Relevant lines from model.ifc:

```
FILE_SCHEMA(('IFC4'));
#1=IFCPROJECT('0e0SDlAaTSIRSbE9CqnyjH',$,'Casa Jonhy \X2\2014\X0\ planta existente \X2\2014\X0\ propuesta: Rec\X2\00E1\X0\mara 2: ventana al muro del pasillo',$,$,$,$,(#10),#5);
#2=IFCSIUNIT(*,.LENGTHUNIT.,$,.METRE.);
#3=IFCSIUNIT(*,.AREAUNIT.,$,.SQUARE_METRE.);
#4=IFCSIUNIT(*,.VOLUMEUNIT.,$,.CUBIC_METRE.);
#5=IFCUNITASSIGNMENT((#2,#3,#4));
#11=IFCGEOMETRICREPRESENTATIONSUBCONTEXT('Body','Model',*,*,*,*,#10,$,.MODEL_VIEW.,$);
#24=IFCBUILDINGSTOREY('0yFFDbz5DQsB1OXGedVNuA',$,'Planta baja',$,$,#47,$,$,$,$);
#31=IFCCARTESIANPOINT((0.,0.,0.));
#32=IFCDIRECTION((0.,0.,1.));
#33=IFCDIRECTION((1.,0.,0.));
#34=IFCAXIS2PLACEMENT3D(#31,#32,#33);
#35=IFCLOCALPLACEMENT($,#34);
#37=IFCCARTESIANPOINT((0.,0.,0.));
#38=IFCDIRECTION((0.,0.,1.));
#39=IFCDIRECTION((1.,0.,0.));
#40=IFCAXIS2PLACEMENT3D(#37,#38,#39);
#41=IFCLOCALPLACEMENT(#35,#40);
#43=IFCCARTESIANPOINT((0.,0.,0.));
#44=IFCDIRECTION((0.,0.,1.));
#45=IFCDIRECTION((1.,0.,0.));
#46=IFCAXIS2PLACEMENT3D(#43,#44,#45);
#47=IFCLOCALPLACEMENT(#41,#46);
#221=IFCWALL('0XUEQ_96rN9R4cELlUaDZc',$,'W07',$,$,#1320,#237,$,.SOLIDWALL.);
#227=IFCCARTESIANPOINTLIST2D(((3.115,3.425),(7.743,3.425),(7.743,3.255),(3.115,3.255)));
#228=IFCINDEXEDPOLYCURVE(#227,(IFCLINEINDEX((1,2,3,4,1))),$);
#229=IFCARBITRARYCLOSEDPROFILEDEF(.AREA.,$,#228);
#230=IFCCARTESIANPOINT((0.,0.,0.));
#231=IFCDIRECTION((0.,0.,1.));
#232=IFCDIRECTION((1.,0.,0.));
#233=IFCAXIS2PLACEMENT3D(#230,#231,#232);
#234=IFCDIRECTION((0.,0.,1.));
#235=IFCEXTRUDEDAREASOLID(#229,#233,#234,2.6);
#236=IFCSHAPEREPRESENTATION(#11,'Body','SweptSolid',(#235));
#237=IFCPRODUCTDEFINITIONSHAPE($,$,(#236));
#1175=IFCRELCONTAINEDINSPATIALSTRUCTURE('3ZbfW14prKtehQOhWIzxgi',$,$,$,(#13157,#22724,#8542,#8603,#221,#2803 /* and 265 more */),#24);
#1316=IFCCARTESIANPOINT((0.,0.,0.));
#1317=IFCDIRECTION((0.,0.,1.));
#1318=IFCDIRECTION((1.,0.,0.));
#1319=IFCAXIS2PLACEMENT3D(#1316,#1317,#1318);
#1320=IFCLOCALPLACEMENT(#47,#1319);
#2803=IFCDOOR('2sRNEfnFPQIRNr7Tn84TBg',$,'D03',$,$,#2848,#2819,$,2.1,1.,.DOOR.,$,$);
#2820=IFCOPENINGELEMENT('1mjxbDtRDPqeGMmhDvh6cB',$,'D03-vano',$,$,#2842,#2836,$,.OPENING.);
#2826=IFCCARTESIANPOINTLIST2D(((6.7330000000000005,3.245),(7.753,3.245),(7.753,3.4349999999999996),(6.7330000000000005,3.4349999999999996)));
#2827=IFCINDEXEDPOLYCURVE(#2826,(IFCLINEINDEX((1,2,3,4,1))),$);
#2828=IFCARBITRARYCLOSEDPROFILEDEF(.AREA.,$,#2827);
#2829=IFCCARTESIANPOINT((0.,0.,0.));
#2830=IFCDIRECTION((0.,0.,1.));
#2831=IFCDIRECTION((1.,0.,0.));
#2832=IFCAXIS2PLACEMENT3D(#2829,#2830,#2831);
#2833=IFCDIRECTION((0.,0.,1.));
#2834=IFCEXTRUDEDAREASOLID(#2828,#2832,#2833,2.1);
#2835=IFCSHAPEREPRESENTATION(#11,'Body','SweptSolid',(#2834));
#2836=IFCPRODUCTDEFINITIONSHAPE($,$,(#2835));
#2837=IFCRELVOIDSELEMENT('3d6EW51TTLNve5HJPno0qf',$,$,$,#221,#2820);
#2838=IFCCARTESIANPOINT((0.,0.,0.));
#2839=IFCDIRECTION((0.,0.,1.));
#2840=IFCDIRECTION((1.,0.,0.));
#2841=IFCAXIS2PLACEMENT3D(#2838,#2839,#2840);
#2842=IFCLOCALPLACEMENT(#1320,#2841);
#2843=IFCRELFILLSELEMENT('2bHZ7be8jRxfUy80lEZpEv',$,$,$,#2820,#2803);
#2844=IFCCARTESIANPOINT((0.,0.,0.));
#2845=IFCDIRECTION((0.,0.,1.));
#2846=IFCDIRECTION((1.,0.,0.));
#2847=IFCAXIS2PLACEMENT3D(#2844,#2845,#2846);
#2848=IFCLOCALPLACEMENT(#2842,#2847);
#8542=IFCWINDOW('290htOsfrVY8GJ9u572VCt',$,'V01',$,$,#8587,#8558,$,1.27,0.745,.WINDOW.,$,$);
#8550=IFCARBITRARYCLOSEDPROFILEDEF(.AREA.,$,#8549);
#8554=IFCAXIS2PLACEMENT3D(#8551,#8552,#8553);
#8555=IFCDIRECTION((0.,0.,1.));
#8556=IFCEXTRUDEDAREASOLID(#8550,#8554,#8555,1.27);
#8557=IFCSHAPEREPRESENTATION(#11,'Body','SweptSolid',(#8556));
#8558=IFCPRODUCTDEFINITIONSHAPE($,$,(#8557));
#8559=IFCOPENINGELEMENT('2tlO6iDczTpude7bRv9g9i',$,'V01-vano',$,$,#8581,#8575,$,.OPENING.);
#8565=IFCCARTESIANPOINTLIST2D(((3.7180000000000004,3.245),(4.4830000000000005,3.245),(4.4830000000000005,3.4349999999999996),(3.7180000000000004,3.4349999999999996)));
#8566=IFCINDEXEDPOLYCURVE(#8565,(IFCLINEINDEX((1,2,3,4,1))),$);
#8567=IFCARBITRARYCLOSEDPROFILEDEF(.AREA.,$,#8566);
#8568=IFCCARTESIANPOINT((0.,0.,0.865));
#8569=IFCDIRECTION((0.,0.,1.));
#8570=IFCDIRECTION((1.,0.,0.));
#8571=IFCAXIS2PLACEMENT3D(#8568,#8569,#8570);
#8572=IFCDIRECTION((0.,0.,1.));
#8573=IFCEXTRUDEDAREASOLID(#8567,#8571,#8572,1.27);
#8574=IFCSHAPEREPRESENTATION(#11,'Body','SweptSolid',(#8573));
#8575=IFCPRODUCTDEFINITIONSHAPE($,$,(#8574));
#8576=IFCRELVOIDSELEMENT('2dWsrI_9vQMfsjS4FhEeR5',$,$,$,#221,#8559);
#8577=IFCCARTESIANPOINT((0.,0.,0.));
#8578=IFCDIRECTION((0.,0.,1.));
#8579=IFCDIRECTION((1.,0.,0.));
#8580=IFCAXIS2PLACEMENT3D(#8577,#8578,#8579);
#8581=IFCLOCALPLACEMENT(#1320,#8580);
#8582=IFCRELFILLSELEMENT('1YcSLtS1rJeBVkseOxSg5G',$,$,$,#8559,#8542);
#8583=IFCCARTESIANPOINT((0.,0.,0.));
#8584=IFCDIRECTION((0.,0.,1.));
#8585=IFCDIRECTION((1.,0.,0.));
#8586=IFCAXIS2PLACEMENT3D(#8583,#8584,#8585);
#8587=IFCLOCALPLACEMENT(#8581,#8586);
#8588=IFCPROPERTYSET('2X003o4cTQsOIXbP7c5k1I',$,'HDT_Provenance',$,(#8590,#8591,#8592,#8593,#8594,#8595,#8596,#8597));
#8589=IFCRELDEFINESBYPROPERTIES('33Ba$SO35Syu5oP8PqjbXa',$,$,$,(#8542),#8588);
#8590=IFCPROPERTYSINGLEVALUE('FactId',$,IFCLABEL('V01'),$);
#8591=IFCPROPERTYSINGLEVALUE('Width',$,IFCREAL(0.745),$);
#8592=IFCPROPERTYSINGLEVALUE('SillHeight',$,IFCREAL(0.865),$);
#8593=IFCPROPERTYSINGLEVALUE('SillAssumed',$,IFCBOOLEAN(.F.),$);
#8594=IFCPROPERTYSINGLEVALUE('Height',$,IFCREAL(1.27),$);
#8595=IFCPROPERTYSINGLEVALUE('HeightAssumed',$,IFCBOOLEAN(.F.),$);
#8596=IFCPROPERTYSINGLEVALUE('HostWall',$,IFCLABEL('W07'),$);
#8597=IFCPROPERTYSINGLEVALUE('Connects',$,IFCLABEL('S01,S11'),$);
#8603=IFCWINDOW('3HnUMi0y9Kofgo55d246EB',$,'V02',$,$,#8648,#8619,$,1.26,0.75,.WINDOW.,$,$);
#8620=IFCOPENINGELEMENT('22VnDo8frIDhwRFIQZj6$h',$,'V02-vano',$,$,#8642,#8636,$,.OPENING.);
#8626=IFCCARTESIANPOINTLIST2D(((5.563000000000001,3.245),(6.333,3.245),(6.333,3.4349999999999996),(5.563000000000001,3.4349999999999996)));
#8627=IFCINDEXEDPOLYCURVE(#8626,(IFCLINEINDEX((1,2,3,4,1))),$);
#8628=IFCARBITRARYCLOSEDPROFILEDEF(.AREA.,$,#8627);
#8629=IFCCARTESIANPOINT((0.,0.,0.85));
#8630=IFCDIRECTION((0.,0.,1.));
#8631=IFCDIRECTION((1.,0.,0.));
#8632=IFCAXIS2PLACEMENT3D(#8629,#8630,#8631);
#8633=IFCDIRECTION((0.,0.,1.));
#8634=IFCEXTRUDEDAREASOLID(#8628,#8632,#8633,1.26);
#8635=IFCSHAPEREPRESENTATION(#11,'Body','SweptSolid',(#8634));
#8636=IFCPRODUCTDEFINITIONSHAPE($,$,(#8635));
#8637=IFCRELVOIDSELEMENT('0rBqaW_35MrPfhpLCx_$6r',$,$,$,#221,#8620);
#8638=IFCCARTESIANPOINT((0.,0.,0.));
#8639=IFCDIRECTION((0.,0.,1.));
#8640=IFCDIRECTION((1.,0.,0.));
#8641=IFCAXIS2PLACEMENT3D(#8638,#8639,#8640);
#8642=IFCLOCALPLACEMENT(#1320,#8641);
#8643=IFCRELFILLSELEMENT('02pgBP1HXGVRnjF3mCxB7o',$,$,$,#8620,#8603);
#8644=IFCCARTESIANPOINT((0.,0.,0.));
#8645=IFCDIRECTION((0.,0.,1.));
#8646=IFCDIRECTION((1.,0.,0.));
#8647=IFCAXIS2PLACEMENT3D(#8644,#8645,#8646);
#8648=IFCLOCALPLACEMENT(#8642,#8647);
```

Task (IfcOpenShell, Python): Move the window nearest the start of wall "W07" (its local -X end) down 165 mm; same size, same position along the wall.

```python
import numpy as np
import ifcopenshell
import ifcopenshell.api.geometry
import ifcopenshell.api.pset
import ifcopenshell.util.element
import ifcopenshell.util.placement
import ifcopenshell.util.unit

model = ifcopenshell.open("model.ifc")
unit_scale = ifcopenshell.util.unit.calculate_unit_scale(model)

window = model.by_guid("290htOsfrVY8GJ9u572VCt")
opening = window.FillsVoids[0].RelatingOpeningElement
dz = -0.165 / unit_scale

shift = np.array([0.0, 0.0, dz])
# The window is placed relative to its opening, so it follows when the opening moves.
matrix = ifcopenshell.util.placement.get_local_placement(opening.ObjectPlacement)
matrix[:3, 3] += shift
ifcopenshell.api.geometry.edit_object_placement(
    model, product=opening, matrix=matrix, is_si=False, should_transform_children=True
)

# Keep the stored heights in step.
pset = model.by_id(ifcopenshell.util.element.get_pset(window, "HDT_Provenance", should_inherit=False)["id"])
ifcopenshell.api.pset.edit_pset(model, pset=pset, properties={
    "SillHeight": model.create_entity("IfcReal", ifcopenshell.util.element.get_pset(window, "HDT_Provenance", "SillHeight") + dz),
})

print(f"moved by {dz * unit_scale:+.3f} m")

model.write("model_edited.ifc")
```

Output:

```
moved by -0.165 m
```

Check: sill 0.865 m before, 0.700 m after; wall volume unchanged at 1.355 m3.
